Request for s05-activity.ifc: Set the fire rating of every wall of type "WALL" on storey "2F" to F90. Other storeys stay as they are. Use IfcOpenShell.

First a look at what the model holds.

```python
import ifcopenshell
import ifcopenshell.util.element

model = ifcopenshell.open("s05-activity.ifc")
print(model.schema)
storey = next(s for s in model.by_type("IfcBuildingStorey") if s.Name == "2F")
walls = [e for e in ifcopenshell.util.element.get_decomposition(storey) if e.is_a("IfcWall")]
seen = {}
for e in walls:
    element_type = ifcopenshell.util.element.get_type(e)
    key = (element_type.Name if element_type != e and element_type else None, ifcopenshell.util.element.get_pset(e, "Pset_WallCommon", "FireRating"))
    seen[key] = seen.get(key, 0) + 1
for (name, value), count in sorted(seen.items(), key=str):
    print(count, "x", name, "|", value)
```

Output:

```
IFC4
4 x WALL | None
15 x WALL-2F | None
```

```python
import ifcopenshell
import ifcopenshell.api.pset
import ifcopenshell.util.element

model = ifcopenshell.open("s05-activity.ifc")

storey = next(s for s in model.by_type("IfcBuildingStorey") if s.Name == "2F")
walls = [e for e in ifcopenshell.util.element.get_decomposition(storey) if e.is_a("IfcWall")]

count = 0
for e in walls:
    element_type = ifcopenshell.util.element.get_type(e)
    if element_type in (None, e) or element_type.Name != "WALL":
        continue
    # add_pset returns the element's existing set when there is one.
    pset = ifcopenshell.api.pset.add_pset(model, product=e, name="Pset_WallCommon")
    ifcopenshell.api.pset.edit_pset(model, pset=pset, properties={"FireRating": "F90"})
    count += 1

print(count, "walls updated")

model.write("s05-activity_v2.ifc")
```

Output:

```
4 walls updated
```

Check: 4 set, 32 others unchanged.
